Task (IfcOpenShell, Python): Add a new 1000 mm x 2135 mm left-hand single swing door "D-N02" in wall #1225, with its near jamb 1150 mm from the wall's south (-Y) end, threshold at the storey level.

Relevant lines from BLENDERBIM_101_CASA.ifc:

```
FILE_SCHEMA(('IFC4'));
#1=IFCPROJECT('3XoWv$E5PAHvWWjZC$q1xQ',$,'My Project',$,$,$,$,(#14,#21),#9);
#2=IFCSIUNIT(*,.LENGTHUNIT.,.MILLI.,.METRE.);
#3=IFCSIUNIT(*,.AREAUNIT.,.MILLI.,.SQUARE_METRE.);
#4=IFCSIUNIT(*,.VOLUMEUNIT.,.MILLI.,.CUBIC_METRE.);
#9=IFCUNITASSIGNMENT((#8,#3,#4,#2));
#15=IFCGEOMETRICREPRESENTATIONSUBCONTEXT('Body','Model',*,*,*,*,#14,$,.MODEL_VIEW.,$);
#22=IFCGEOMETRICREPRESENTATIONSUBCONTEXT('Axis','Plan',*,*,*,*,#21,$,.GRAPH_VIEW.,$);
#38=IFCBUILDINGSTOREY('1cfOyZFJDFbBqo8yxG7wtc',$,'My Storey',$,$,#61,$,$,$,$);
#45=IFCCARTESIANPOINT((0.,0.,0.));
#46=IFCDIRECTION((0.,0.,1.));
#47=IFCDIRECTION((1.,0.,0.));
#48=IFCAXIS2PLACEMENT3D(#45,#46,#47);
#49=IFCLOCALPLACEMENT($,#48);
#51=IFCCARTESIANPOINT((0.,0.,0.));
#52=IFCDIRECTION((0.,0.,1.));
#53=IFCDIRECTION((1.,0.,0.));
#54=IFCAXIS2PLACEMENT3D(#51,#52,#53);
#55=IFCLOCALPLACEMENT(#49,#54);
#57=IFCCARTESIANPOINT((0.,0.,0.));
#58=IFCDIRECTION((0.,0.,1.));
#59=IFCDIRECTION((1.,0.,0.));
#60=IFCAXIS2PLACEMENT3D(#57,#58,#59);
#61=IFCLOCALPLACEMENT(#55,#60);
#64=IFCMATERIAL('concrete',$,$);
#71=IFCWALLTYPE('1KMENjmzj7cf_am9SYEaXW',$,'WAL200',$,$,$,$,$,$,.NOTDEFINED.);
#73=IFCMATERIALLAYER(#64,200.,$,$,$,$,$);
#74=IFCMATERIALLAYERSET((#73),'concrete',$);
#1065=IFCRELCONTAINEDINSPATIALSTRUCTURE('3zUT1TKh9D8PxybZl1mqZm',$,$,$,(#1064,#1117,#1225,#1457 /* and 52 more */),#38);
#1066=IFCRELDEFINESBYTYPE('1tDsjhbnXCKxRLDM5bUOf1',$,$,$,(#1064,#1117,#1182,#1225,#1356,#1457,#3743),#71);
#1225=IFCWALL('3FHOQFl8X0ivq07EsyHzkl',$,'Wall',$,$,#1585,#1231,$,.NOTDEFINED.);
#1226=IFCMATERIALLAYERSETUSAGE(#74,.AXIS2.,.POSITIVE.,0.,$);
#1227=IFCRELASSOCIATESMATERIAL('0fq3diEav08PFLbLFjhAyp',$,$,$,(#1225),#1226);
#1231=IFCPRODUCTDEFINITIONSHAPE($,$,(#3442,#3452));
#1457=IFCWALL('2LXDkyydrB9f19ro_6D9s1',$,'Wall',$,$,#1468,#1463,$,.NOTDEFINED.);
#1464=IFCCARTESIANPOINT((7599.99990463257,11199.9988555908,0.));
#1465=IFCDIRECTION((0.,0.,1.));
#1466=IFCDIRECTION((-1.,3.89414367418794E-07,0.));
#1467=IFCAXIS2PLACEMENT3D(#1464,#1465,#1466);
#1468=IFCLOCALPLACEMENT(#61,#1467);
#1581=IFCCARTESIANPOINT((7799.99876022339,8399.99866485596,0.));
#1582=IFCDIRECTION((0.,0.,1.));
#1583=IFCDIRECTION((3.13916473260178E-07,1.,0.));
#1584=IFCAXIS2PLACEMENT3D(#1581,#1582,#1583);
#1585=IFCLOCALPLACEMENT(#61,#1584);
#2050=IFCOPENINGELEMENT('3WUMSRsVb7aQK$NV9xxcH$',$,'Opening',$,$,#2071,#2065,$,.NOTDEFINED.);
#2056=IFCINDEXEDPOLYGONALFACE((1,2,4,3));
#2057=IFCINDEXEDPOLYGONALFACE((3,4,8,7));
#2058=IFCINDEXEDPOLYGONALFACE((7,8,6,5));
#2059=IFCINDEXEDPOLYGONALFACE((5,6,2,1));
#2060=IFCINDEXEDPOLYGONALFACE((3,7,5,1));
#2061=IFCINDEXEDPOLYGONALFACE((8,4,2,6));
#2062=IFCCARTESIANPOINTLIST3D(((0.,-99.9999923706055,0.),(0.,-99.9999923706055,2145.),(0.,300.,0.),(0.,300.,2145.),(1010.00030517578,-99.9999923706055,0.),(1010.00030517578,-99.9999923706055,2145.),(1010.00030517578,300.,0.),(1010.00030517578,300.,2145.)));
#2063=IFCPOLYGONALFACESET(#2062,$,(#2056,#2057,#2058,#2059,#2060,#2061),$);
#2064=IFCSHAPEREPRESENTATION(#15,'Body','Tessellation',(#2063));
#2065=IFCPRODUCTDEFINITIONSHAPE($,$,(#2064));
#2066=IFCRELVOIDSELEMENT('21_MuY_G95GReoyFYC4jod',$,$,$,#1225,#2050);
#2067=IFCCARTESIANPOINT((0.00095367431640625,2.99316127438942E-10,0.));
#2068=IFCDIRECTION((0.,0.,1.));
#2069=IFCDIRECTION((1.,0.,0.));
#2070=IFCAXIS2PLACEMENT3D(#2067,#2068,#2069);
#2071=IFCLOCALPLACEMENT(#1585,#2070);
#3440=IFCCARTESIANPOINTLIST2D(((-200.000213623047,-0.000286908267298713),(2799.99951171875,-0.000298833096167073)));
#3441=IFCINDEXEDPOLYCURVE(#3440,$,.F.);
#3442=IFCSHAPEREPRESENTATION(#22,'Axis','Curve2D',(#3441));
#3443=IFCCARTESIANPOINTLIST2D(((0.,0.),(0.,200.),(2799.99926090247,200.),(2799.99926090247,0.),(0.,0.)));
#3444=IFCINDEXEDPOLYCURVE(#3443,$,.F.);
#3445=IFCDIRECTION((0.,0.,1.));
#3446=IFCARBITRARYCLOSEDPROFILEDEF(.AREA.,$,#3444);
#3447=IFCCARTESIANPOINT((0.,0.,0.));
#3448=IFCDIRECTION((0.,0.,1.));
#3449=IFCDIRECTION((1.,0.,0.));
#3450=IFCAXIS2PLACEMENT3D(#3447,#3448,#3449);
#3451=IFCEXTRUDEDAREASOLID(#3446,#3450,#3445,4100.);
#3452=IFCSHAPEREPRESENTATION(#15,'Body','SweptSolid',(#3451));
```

```python
import numpy as np
import ifcopenshell
import ifcopenshell.api.feature
import ifcopenshell.api.geometry
import ifcopenshell.api.root
import ifcopenshell.api.spatial
import ifcopenshell.geom
import ifcopenshell.util.element
import ifcopenshell.util.placement
import ifcopenshell.util.representation
import ifcopenshell.util.shape
import ifcopenshell.util.unit

model = ifcopenshell.open("BLENDERBIM_101_CASA.ifc")
unit_scale = ifcopenshell.util.unit.calculate_unit_scale(model)
settings = ifcopenshell.geom.settings()


def volume(element):
    """Net volume in cubic metres, openings subtracted."""
    shape = ifcopenshell.geom.create_shape(settings, element)
    return ifcopenshell.util.shape.get_volume(shape.geometry)


wall = model.by_guid("3FHOQFl8X0ivq07EsyHzkl")
storey = ifcopenshell.util.element.get_container(wall, ifc_class="IfcBuildingStorey")
context = ifcopenshell.util.representation.get_context(model, "Model", "Body", "MODEL_VIEW")
before = volume(wall)

width, height, from_end, sill = 1, 2.135, 1.15, 0.0  # metres

# The wall runs along its own X axis, and the end named is its -X end.
wall_shape = ifcopenshell.geom.create_shape(settings, wall)
x, y, z = ifcopenshell.util.shape.get_vertices(wall_shape.geometry).T
start = x.min() + from_end
face, thickness = float(y.min()), float(y.max() - y.min())
wall_matrix = ifcopenshell.util.placement.get_local_placement(wall.ObjectPlacement)
level = ifcopenshell.util.placement.get_local_placement(storey.ObjectPlacement)[2, 3]


def in_wall(x, y):
    """Placement at x, y metres in the wall's axes, at sill height."""
    matrix = wall_matrix.copy()
    matrix[:, 3] = wall_matrix @ np.array([x / unit_scale, y / unit_scale, 0.0, 1.0])
    matrix[2, 3] = level + sill / unit_scale
    return matrix


# Opening: a box that overshoots both wall faces by 50 mm.
opening = ifcopenshell.api.root.create_entity(model, ifc_class="IfcOpeningElement", predefined_type="OPENING")
box = ifcopenshell.api.geometry.add_wall_representation(
    model, context=context, length=width, height=height, thickness=thickness + 0.1
)
ifcopenshell.api.geometry.assign_representation(model, product=opening, representation=box)
ifcopenshell.api.geometry.edit_object_placement(model, product=opening, matrix=in_wall(start, face - 0.05), is_si=False)
ifcopenshell.api.feature.add_feature(model, feature=opening, element=wall)

door = ifcopenshell.api.root.create_entity(model, ifc_class="IfcDoor", name="D-N02", predefined_type="DOOR")
door.OverallWidth, door.OverallHeight = width / unit_scale, height / unit_scale
door.OperationType = "SINGLE_SWING_LEFT"
body = ifcopenshell.api.geometry.add_door_representation(
    model,
    context=context,
    overall_width=door.OverallWidth,
    overall_height=door.OverallHeight,
    operation_type="SINGLE_SWING_LEFT",
    lining_properties={"LiningDepth": thickness / unit_scale, "ThresholdDepth": thickness / unit_scale},
)
ifcopenshell.api.geometry.assign_representation(model, product=door, representation=body)
ifcopenshell.api.spatial.assign_container(model, products=[door], relating_structure=storey)
ifcopenshell.api.feature.add_filling(model, opening=opening, element=door)

# The lining spans the wall, so the door starts at the wall face.
ifcopenshell.api.geometry.edit_object_placement(model, product=door, matrix=in_wall(start, face), is_si=False)

after = volume(wall)

print(f"wall volume {before:.3f} -> {after:.3f} m3")

model.write("BLENDERBIM_101_CASA-out.ifc")
```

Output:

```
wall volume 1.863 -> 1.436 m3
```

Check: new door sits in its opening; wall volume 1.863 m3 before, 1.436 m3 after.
